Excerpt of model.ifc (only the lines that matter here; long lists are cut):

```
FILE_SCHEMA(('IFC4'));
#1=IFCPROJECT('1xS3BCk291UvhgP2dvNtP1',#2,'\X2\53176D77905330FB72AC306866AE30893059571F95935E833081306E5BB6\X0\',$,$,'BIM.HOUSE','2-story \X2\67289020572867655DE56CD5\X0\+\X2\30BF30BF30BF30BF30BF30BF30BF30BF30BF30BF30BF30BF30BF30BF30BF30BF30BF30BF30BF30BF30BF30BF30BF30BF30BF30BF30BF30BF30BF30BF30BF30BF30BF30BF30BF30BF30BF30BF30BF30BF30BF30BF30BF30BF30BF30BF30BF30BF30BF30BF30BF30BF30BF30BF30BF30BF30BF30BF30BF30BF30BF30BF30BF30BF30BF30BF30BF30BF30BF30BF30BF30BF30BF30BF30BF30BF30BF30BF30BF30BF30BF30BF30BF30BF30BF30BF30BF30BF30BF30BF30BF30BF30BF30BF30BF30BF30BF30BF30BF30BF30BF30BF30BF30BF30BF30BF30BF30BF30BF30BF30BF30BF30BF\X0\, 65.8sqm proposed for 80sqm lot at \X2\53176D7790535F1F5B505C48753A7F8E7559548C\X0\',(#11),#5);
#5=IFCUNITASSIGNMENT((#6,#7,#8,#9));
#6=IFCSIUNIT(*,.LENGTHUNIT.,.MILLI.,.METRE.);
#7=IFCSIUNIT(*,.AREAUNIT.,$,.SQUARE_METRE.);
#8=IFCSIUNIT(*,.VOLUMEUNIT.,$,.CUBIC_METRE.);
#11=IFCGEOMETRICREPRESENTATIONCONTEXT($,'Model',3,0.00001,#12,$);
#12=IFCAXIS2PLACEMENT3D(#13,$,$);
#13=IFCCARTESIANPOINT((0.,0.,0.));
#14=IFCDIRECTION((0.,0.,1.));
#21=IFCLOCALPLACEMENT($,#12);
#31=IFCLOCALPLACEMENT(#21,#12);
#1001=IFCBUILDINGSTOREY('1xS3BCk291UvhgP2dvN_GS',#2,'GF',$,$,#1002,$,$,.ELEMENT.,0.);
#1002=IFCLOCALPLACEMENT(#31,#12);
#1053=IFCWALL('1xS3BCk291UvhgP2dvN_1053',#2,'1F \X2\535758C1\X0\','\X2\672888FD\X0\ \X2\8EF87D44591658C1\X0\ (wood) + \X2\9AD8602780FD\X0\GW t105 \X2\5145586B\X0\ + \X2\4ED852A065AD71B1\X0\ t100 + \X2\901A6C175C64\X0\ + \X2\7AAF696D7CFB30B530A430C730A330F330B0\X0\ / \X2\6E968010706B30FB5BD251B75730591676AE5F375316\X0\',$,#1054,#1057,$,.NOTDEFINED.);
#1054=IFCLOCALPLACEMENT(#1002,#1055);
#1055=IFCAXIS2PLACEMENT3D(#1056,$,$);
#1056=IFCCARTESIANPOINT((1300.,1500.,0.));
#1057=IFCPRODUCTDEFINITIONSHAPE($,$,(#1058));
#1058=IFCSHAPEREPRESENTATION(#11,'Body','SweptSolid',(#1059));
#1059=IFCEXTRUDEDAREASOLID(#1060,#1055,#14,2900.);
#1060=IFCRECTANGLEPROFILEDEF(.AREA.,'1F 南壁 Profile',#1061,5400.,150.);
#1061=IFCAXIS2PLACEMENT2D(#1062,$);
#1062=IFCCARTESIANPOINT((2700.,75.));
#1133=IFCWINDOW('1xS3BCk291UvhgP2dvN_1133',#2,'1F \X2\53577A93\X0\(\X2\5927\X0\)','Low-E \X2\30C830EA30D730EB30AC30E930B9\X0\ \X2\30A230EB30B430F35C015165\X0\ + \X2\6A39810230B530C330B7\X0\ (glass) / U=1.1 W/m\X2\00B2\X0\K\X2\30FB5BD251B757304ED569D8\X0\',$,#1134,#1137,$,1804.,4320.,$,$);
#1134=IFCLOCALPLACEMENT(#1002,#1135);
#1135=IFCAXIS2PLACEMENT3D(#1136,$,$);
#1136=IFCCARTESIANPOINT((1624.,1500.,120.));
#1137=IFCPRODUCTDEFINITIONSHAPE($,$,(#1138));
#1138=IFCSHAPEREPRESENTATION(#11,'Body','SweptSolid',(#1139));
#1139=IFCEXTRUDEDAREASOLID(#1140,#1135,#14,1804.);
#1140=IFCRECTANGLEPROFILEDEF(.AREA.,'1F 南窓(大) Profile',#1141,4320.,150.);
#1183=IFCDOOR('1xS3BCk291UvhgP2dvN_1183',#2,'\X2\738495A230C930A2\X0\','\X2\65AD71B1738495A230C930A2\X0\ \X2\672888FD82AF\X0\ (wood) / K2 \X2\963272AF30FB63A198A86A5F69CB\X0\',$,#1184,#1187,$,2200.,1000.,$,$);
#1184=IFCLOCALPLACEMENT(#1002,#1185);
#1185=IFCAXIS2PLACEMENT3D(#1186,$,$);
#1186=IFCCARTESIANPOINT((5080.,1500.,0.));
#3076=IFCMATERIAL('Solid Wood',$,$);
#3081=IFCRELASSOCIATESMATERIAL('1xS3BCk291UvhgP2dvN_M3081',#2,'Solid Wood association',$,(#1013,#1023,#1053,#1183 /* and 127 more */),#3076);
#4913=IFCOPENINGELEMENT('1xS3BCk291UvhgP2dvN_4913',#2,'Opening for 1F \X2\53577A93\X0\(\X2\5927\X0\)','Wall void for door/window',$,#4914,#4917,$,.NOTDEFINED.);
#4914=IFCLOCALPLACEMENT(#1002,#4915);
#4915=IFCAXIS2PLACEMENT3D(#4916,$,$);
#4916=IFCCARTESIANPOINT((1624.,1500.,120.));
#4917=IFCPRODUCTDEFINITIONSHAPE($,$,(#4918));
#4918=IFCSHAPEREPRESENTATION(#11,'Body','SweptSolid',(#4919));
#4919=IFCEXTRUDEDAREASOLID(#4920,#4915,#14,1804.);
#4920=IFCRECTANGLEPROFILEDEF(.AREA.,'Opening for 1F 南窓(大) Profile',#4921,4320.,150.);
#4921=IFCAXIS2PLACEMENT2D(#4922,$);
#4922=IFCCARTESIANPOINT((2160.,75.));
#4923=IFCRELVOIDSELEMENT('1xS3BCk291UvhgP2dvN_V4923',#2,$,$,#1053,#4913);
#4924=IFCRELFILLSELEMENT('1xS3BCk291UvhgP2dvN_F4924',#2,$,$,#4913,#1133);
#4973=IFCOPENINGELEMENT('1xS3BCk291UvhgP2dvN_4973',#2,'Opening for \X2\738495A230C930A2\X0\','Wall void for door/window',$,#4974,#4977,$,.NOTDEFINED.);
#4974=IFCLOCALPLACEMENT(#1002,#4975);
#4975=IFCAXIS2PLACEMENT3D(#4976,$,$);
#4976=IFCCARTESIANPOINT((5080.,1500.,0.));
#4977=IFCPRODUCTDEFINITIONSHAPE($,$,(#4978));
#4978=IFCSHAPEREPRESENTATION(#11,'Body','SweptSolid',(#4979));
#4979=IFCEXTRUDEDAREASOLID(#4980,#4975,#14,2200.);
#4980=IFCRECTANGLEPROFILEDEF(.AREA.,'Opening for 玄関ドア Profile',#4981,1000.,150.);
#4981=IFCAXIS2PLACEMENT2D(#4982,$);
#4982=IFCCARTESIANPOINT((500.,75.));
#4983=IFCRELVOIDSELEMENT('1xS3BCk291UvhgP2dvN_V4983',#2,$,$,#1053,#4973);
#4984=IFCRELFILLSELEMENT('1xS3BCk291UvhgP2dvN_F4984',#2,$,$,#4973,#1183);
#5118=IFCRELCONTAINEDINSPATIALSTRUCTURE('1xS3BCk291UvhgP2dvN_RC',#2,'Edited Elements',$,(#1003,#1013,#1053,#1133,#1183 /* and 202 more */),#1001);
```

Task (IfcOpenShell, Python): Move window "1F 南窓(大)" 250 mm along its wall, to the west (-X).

```python
import ifcopenshell
import ifcopenshell.api.geometry
import ifcopenshell.util.placement
import ifcopenshell.util.unit

model = ifcopenshell.open("model.ifc")
unit_scale = ifcopenshell.util.unit.calculate_unit_scale(model)

window = model.by_guid("1xS3BCk291UvhgP2dvN_1133")
opening = window.FillsVoids[0].RelatingOpeningElement
wall = opening.VoidsElements[0].RelatingBuildingElement

wall_matrix = ifcopenshell.util.placement.get_local_placement(wall.ObjectPlacement)
shift = wall_matrix[:3, 0] * -0.25 / unit_scale
before = ifcopenshell.util.placement.get_local_placement(window.ObjectPlacement)[:3, 3].copy()

# The window is not placed relative to its opening, so move both.
for product in (opening, window):
    matrix = ifcopenshell.util.placement.get_local_placement(product.ObjectPlacement)
    matrix[:3, 3] += shift
    ifcopenshell.api.geometry.edit_object_placement(model, product=product, matrix=matrix, is_si=False)

after = ifcopenshell.util.placement.get_local_placement(window.ObjectPlacement)[:3, 3]
print("window moved by", (after - before).round(3) + 0.0)

model.write("model-out.ifc")
```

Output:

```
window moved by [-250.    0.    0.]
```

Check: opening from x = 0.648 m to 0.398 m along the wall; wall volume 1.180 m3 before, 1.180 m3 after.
